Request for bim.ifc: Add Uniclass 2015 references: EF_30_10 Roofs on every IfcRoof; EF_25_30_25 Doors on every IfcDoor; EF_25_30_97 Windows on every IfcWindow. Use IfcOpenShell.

First a look at what the model holds.

```python
import ifcopenshell

model = ifcopenshell.open("bim.ifc")
print(model.schema)
print("classifications:", [c.Name for c in model.by_type("IfcClassification")])
for ifc_class in ("IfcDoor", "IfcRoof", "IfcStair", "IfcWall", "IfcWindow"):
    print(ifc_class, len(model.by_type(ifc_class)))
```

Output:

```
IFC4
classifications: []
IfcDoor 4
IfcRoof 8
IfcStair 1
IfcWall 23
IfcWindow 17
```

```python
import ifcopenshell
import ifcopenshell.api.classification

model = ifcopenshell.open("bim.ifc")

system = ifcopenshell.api.classification.add_classification(model, classification="Uniclass 2015")

codes = {
    "IfcRoof": ("EF_30_10", "Roofs"),
    "IfcDoor": ("EF_25_30_25", "Doors"),
    "IfcWindow": ("EF_25_30_97", "Windows"),
}
for ifc_class, (code, name) in codes.items():
    products = model.by_type(ifc_class)
    ifcopenshell.api.classification.add_reference(
        model, products=products, classification=system, identification=code, name=name
    )
    print(code, len(products))

model.write("bim_rev.ifc")
```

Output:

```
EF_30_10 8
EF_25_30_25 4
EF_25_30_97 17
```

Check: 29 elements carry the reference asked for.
